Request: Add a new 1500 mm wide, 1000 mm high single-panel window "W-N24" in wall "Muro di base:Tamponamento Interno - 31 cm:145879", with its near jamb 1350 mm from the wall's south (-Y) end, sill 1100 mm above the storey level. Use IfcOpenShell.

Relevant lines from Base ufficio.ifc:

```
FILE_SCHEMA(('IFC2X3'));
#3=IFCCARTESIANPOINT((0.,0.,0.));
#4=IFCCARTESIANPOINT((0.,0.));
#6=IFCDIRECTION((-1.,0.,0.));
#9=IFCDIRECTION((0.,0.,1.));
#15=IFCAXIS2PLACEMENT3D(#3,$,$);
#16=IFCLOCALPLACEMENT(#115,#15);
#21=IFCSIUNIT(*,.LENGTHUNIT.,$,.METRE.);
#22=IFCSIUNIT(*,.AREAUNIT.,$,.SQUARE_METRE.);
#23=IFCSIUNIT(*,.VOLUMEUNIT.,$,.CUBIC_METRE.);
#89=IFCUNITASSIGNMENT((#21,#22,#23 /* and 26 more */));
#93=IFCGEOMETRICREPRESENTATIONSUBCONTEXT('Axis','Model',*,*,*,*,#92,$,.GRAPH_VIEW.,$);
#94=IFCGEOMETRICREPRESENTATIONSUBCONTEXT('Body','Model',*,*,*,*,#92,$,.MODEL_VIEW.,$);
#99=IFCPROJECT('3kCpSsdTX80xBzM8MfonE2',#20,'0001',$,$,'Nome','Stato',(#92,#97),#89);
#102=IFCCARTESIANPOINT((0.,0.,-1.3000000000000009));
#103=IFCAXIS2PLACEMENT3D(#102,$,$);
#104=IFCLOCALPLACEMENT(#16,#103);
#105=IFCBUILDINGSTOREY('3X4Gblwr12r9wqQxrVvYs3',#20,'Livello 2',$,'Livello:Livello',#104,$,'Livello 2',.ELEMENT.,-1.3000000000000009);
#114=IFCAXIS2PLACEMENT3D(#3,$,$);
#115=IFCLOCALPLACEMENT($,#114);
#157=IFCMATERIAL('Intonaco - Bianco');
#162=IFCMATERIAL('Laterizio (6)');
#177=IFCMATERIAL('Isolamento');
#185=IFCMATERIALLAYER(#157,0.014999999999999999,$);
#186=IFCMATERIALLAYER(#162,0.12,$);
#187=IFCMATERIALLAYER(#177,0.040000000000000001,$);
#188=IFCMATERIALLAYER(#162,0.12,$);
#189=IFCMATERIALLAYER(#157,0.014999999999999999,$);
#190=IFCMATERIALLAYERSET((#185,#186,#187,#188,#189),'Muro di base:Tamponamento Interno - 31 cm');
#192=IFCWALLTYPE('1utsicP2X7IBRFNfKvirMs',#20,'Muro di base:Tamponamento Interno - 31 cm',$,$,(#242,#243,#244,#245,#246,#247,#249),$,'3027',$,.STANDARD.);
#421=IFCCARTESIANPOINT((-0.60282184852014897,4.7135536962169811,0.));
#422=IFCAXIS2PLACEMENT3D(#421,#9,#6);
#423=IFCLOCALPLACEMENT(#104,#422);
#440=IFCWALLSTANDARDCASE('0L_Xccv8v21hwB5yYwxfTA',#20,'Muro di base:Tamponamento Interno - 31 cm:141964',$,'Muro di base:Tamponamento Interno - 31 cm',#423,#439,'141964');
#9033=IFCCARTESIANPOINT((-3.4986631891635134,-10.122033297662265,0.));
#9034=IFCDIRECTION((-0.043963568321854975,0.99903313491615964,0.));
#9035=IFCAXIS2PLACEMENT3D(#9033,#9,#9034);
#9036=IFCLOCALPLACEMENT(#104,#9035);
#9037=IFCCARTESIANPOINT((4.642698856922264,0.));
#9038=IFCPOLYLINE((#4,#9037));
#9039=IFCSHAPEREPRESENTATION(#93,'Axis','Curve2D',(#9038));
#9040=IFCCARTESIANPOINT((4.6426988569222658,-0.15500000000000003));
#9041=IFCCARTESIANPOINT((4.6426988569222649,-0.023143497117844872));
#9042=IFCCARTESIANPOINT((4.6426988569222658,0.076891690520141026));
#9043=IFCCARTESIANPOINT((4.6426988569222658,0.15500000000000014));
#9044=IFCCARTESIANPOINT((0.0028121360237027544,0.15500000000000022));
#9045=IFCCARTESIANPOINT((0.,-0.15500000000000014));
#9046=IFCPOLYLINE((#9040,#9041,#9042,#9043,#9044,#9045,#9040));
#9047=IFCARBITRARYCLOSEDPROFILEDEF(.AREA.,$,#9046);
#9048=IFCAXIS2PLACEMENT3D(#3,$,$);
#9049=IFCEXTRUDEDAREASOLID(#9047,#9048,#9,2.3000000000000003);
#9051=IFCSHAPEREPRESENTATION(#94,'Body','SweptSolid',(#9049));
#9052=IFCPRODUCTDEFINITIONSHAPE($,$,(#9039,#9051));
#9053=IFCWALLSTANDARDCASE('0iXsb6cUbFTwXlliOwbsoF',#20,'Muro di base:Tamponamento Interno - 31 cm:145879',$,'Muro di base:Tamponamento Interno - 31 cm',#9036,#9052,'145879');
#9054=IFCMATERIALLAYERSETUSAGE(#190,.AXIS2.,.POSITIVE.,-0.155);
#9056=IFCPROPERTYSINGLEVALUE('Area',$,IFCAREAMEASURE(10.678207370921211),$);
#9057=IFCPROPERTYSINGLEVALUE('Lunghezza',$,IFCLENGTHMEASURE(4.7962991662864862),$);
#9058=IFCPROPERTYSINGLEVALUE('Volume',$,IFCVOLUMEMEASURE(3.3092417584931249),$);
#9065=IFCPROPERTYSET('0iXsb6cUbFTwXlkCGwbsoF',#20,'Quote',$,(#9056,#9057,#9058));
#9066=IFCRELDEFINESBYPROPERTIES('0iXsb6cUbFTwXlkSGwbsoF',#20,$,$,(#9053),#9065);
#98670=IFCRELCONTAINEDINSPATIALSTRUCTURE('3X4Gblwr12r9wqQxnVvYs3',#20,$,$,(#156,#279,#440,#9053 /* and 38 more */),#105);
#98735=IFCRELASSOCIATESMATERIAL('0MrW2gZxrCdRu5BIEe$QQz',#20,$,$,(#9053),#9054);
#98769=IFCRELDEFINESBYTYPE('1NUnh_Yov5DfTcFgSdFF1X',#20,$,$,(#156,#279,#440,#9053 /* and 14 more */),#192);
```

```python
import numpy as np
import ifcopenshell
import ifcopenshell.api.feature
import ifcopenshell.api.geometry
import ifcopenshell.api.pset
import ifcopenshell.api.root
import ifcopenshell.api.spatial
import ifcopenshell.api.type
import ifcopenshell.geom
import ifcopenshell.util.element
import ifcopenshell.util.placement
import ifcopenshell.util.representation
import ifcopenshell.util.shape
import ifcopenshell.util.unit

model = ifcopenshell.open("Base ufficio.ifc")
unit_scale = ifcopenshell.util.unit.calculate_unit_scale(model)
area_scale = ifcopenshell.util.unit.calculate_unit_scale(model, "AREAUNIT")
volume_scale = ifcopenshell.util.unit.calculate_unit_scale(model, "VOLUMEUNIT")
settings = ifcopenshell.geom.settings()


def volume(element):
    """Net volume in cubic metres, openings subtracted."""
    shape = ifcopenshell.geom.create_shape(settings, element)
    return ifcopenshell.util.shape.get_volume(shape.geometry)


wall = model.by_guid("0iXsb6cUbFTwXlliOwbsoF")
storey = ifcopenshell.util.element.get_container(wall, ifc_class="IfcBuildingStorey")
context = ifcopenshell.util.representation.get_context(model, "Model", "Body", "MODEL_VIEW")
before = volume(wall)

width, height, from_end, sill = 1.5, 1, 1.35, 1.1  # metres

# The wall runs along its own X axis, and the end named is its -X end.
wall_shape = ifcopenshell.geom.create_shape(settings, wall)
x, y, z = ifcopenshell.util.shape.get_vertices(wall_shape.geometry).T
start = x.min() + from_end
face, thickness = float(y.min()), float(y.max() - y.min())
wall_matrix = ifcopenshell.util.placement.get_local_placement(wall.ObjectPlacement)
level = ifcopenshell.util.placement.get_local_placement(storey.ObjectPlacement)[2, 3]


def in_wall(x, y):
    """Placement at x, y metres in the wall's axes, at sill height."""
    matrix = wall_matrix.copy()
    matrix[:, 3] = wall_matrix @ np.array([x / unit_scale, y / unit_scale, 0.0, 1.0])
    matrix[2, 3] = level + sill / unit_scale
    return matrix


# Opening: a box that overshoots both wall faces by 50 mm.
opening = ifcopenshell.api.root.create_entity(model, ifc_class="IfcOpeningElement")
box = ifcopenshell.api.geometry.add_wall_representation(
    model, context=context, length=width, height=height, thickness=thickness + 0.1
)
ifcopenshell.api.geometry.assign_representation(model, product=opening, representation=box)
ifcopenshell.api.geometry.edit_object_placement(model, product=opening, matrix=in_wall(start, face - 0.05), is_si=False)
ifcopenshell.api.feature.add_feature(model, feature=opening, element=wall)

window = ifcopenshell.api.root.create_entity(model, ifc_class="IfcWindow", name="W-N24")
window.OverallWidth, window.OverallHeight = width / unit_scale, height / unit_scale
body = ifcopenshell.api.geometry.add_window_representation(
    model,
    context=context,
    overall_width=window.OverallWidth,
    overall_height=window.OverallHeight,
    partition_type="SINGLE_PANEL",
)
ifcopenshell.api.geometry.assign_representation(model, product=window, representation=body)
ifcopenshell.api.spatial.assign_container(model, products=[window], relating_structure=storey)
fills = ifcopenshell.api.feature.add_filling(model, opening=opening, element=window)
fills.OwnerHistory = window.OwnerHistory  # required in IFC2X3

# IFC2X3 keeps the operation on the window style.
style = ifcopenshell.api.root.create_entity(model, ifc_class="IfcWindowStyle", name="W-N24")
style.OperationType, style.ConstructionType = "SINGLE_PANEL", "NOTDEFINED"
style.ParameterTakesPrecedence = style.Sizeable = False
ifcopenshell.api.type.assign_type(model, related_objects=[window], relating_type=style)

# Centre the window in the wall's thickness.
ifcopenshell.api.geometry.edit_object_placement(model, product=window, matrix=in_wall(start, face), is_si=False)
window_shape = ifcopenshell.geom.create_shape(settings, window)
depth = ifcopenshell.util.shape.get_vertices(window_shape.geometry)[:, 1]
offset = face + thickness / 2 - (depth.min() + depth.max()) / 2
ifcopenshell.api.geometry.edit_object_placement(model, product=window, matrix=in_wall(start, offset), is_si=False)

after = volume(wall)

# Update the wall's stored quantities.
pset = model.by_id(ifcopenshell.util.element.get_pset(wall, "Quote", should_inherit=False)["id"])
ifcopenshell.api.pset.edit_pset(model, pset=pset, properties={
    "Area": model.create_entity("IfcAreaMeasure", after / thickness / area_scale),
    "Volume": model.create_entity("IfcVolumeMeasure", after / volume_scale),
})

print(f"wall volume {before:.3f} -> {after:.3f} m3")

model.write("Base ufficio_v2.ifc")
```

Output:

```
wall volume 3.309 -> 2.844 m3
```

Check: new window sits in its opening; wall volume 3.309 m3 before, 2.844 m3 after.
